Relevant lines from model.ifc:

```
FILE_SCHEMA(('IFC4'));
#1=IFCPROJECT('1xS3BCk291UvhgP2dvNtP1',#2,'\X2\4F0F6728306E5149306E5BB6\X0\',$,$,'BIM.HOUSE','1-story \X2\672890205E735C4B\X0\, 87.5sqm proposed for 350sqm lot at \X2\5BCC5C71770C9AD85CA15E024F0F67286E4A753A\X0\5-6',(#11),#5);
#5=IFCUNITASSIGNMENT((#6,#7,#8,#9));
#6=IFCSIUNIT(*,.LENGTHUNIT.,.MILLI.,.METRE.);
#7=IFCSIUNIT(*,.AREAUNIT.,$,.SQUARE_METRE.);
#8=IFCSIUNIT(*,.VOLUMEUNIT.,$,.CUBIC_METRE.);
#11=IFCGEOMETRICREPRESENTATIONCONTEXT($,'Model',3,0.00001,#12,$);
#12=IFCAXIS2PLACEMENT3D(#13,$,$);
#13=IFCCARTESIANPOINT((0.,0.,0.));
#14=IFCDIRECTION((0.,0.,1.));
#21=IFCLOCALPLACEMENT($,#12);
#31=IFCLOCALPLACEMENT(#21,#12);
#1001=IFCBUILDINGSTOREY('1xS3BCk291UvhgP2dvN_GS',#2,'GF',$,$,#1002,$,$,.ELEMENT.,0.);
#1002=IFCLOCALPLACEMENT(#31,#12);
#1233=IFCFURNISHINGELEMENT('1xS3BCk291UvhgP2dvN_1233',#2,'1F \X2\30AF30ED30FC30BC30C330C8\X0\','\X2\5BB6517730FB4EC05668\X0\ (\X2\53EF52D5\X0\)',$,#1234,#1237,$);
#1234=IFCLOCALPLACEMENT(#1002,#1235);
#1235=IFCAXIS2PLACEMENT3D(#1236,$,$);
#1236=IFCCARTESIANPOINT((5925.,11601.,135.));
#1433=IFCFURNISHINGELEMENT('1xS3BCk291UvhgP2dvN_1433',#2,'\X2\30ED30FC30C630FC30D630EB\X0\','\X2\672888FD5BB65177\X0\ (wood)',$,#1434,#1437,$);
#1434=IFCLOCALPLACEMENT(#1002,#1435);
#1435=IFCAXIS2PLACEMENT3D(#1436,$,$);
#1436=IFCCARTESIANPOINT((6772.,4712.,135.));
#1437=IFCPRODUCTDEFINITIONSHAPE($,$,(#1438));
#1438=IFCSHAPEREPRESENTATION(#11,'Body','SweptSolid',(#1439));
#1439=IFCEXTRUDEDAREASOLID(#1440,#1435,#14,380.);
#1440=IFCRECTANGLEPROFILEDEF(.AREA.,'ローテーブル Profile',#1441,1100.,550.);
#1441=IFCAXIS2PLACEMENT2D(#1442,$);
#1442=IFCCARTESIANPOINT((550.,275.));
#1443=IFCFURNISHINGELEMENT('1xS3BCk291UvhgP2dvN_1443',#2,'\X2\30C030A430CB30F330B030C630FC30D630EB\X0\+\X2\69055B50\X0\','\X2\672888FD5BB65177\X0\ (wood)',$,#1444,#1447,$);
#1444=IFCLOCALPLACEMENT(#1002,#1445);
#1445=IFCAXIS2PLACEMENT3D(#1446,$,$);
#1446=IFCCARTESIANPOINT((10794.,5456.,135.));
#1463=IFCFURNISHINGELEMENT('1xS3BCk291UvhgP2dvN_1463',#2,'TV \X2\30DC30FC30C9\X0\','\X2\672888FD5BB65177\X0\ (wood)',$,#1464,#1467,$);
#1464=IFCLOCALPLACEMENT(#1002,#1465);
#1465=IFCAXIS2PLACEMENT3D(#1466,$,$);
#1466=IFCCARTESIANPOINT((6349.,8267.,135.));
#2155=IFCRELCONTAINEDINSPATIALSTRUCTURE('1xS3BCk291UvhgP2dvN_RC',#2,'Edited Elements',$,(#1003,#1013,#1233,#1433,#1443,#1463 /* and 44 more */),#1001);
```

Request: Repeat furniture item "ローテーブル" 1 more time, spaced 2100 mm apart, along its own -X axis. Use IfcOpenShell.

```python
import ifcopenshell
import ifcopenshell.api.geometry
import ifcopenshell.api.root
import ifcopenshell.util.element
import ifcopenshell.util.placement
import ifcopenshell.util.unit

model = ifcopenshell.open("model.ifc")
unit_scale = ifcopenshell.util.unit.calculate_unit_scale(model)


def reuse_history(source, copy):
    """copy_class also copies each property set's owner history, people and application; keep the originals."""
    for rel in copy.IsDefinedBy:
        if rel.is_a("IfcRelDefinesByProperties") and (history := rel.RelatingPropertyDefinition.OwnerHistory):
            rel.RelatingPropertyDefinition.OwnerHistory = source.OwnerHistory
            ifcopenshell.util.element.remove_deep2(model, history)


source = model.by_guid("1xS3BCk291UvhgP2dvN_1433")
base = ifcopenshell.util.placement.get_local_placement(source.ObjectPlacement)
step = -base[:3, 0] * 2.1 / unit_scale

for i in range(1, 2):
    copy = ifcopenshell.api.root.copy_class(model, product=source)
    copy.Representation = ifcopenshell.util.element.copy_deep(
        model, source.Representation, exclude=["IfcGeometricRepresentationContext", "IfcRepresentationMap"]
    )
    reuse_history(source, copy)
    matrix = base.copy()
    matrix[:3, 3] += i * step
    print("added at", matrix[:3, 3].round(3) + 0.0)
    ifcopenshell.api.geometry.edit_object_placement(model, product=copy, matrix=matrix, is_si=False)

model.write("model_rev.ifc")
```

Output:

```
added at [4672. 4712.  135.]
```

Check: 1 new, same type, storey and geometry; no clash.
